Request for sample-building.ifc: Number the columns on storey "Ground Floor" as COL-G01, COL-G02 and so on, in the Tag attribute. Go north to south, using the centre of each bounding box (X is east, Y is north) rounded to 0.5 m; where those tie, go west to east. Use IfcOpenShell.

First a look at what the model holds.

```python
import ifcopenshell
import ifcopenshell.util.element
import ifcopenshell.util.placement

model = ifcopenshell.open("sample-building.ifc")
print(model.schema)
storey = next(s for s in model.by_type("IfcBuildingStorey") if s.Name == "Ground Floor")
columns = [e for e in ifcopenshell.util.element.get_decomposition(storey) if e.is_a("IfcColumn")]
for e in sorted(columns, key=lambda e: e.id()):
    origin = ifcopenshell.util.placement.get_local_placement(e.ObjectPlacement)[:3, 3]
    print(e.id(), e.Tag, e.Name, origin.round(2) + 0.0, sep=" | ")
```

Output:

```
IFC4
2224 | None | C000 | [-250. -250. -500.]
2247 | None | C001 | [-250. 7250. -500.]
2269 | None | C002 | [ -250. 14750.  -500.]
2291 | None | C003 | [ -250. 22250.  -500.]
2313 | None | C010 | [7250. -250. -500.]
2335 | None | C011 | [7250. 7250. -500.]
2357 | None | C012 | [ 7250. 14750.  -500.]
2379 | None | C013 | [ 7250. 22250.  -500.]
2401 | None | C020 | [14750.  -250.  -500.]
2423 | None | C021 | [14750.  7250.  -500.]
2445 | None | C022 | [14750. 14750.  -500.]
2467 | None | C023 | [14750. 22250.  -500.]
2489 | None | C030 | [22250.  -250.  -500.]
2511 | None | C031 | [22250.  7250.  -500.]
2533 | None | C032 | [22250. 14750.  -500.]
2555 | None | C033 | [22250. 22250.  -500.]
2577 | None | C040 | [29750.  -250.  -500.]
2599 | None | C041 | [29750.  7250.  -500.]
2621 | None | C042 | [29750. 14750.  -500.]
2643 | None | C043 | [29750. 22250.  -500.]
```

```python
import ifcopenshell
import ifcopenshell.geom
import ifcopenshell.util.element
import ifcopenshell.util.shape

model = ifcopenshell.open("sample-building.ifc")
settings = ifcopenshell.geom.settings()
settings.set("use-world-coords", True)


def centre(element):
    shape = ifcopenshell.geom.create_shape(settings, element)
    return ifcopenshell.util.shape.get_bbox_centroid(shape.geometry)


storey = next(s for s in model.by_type("IfcBuildingStorey") if s.Name == "Ground Floor")
columns = [e for e in ifcopenshell.util.element.get_decomposition(storey) if e.is_a("IfcColumn")]

# Insertion points can sit at a corner or the storey origin, so sort by the geometry (in metres).
centres = {e: centre(e) for e in columns}
columns.sort(key=lambda e: (-round(centres[e][1] / 0.5), centres[e][0]))

for i, e in enumerate(columns, start=1):
    number = f"COL-G{i:02d}"
    e.Tag = number
    print(e.id(), number)

model.write("sample-building-out.ifc")
```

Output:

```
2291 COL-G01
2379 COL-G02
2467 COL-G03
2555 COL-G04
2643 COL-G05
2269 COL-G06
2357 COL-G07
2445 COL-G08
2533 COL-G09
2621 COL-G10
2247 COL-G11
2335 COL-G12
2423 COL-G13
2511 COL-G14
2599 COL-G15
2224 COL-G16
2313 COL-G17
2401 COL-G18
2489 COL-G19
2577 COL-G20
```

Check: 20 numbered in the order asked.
